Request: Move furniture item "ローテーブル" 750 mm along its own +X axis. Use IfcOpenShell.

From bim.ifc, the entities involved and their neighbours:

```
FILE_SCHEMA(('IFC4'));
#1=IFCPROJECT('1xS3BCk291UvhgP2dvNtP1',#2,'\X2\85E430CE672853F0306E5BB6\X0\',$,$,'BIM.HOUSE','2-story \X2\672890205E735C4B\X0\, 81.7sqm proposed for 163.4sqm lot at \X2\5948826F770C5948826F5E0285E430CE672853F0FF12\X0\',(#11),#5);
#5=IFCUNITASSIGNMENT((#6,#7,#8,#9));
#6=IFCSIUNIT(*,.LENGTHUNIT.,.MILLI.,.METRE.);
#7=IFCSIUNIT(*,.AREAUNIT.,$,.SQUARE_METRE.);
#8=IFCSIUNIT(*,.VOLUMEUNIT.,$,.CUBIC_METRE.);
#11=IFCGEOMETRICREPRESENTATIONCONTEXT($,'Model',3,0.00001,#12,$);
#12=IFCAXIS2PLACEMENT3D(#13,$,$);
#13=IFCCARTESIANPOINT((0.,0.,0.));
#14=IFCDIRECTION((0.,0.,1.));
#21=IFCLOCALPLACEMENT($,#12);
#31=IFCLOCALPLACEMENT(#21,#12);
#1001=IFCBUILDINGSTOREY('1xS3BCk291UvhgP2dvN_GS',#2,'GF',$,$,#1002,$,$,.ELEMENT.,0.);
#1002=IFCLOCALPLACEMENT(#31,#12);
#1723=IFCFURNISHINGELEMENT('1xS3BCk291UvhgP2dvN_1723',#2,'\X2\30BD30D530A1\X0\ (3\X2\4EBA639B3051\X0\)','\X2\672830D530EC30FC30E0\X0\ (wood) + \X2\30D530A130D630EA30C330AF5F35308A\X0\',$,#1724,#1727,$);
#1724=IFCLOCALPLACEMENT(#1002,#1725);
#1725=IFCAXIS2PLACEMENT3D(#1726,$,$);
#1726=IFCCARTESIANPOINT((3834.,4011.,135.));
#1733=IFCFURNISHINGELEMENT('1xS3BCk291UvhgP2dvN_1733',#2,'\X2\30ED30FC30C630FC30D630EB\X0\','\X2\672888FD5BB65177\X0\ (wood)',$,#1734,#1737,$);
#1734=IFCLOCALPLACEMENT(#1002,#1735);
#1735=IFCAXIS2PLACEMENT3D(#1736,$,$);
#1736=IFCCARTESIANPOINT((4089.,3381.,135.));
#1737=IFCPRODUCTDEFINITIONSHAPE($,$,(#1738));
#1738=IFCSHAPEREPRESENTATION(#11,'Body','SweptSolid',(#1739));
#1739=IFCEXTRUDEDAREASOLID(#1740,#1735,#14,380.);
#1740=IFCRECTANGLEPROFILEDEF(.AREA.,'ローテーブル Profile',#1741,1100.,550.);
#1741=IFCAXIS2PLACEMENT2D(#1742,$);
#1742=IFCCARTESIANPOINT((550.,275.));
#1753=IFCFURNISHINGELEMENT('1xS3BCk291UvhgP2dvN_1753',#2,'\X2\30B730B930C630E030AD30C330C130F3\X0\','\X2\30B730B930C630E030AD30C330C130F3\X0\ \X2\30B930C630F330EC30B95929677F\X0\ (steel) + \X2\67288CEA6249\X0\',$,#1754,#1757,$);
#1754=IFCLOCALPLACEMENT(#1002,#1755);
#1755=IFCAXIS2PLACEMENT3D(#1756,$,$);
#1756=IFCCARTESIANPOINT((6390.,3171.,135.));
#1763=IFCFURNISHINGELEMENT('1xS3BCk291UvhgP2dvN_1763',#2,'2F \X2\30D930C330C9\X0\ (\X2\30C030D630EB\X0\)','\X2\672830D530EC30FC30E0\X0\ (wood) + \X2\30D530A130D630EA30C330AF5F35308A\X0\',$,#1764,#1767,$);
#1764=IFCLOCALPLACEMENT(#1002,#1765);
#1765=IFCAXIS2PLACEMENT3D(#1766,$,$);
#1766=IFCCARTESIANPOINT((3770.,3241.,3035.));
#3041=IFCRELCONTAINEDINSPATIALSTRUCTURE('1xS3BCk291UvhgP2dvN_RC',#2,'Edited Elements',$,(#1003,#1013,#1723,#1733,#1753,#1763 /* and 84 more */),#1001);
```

```python
import ifcopenshell
import ifcopenshell.api.geometry
import ifcopenshell.util.placement
import ifcopenshell.util.unit

model = ifcopenshell.open("bim.ifc")
unit_scale = ifcopenshell.util.unit.calculate_unit_scale(model)

item = model.by_guid("1xS3BCk291UvhgP2dvN_1733")
matrix = ifcopenshell.util.placement.get_local_placement(item.ObjectPlacement)
matrix[:3, 3] += matrix[:3, 0] * 0.75 / unit_scale
ifcopenshell.api.geometry.edit_object_placement(model, product=item, matrix=matrix, is_si=False)

print(ifcopenshell.util.placement.get_local_placement(item.ObjectPlacement).round(3) + 0.0)

model.write("bim_edited.ifc")
```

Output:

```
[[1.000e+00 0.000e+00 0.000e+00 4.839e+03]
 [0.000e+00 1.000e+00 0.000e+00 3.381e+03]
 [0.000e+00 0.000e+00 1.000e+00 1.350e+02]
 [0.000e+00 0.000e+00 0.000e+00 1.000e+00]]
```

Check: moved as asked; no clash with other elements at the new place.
